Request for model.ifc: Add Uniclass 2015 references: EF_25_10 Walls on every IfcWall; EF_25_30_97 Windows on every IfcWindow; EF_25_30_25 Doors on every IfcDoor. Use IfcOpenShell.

First a look at what the model holds.

```python
import ifcopenshell

model = ifcopenshell.open("model.ifc")
print(model.schema)
print("classifications:", [c.Name for c in model.by_type("IfcClassification")])
for ifc_class in ("IfcDoor", "IfcRoof", "IfcStair", "IfcWall", "IfcWindow"):
    print(ifc_class, len(model.by_type(ifc_class)))
```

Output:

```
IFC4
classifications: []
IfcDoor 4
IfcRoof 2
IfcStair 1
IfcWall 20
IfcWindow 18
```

```python
import ifcopenshell
import ifcopenshell.api.classification

model = ifcopenshell.open("model.ifc")

system = ifcopenshell.api.classification.add_classification(model, classification="Uniclass 2015")

codes = {
    "IfcWall": ("EF_25_10", "Walls"),
    "IfcWindow": ("EF_25_30_97", "Windows"),
    "IfcDoor": ("EF_25_30_25", "Doors"),
}
for ifc_class, (code, name) in codes.items():
    products = model.by_type(ifc_class)
    ifcopenshell.api.classification.add_reference(
        model, products=products, classification=system, identification=code, name=name
    )
    print(code, len(products))

model.write("model_edited.ifc")
```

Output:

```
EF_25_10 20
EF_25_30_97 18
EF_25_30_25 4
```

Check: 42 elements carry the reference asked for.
